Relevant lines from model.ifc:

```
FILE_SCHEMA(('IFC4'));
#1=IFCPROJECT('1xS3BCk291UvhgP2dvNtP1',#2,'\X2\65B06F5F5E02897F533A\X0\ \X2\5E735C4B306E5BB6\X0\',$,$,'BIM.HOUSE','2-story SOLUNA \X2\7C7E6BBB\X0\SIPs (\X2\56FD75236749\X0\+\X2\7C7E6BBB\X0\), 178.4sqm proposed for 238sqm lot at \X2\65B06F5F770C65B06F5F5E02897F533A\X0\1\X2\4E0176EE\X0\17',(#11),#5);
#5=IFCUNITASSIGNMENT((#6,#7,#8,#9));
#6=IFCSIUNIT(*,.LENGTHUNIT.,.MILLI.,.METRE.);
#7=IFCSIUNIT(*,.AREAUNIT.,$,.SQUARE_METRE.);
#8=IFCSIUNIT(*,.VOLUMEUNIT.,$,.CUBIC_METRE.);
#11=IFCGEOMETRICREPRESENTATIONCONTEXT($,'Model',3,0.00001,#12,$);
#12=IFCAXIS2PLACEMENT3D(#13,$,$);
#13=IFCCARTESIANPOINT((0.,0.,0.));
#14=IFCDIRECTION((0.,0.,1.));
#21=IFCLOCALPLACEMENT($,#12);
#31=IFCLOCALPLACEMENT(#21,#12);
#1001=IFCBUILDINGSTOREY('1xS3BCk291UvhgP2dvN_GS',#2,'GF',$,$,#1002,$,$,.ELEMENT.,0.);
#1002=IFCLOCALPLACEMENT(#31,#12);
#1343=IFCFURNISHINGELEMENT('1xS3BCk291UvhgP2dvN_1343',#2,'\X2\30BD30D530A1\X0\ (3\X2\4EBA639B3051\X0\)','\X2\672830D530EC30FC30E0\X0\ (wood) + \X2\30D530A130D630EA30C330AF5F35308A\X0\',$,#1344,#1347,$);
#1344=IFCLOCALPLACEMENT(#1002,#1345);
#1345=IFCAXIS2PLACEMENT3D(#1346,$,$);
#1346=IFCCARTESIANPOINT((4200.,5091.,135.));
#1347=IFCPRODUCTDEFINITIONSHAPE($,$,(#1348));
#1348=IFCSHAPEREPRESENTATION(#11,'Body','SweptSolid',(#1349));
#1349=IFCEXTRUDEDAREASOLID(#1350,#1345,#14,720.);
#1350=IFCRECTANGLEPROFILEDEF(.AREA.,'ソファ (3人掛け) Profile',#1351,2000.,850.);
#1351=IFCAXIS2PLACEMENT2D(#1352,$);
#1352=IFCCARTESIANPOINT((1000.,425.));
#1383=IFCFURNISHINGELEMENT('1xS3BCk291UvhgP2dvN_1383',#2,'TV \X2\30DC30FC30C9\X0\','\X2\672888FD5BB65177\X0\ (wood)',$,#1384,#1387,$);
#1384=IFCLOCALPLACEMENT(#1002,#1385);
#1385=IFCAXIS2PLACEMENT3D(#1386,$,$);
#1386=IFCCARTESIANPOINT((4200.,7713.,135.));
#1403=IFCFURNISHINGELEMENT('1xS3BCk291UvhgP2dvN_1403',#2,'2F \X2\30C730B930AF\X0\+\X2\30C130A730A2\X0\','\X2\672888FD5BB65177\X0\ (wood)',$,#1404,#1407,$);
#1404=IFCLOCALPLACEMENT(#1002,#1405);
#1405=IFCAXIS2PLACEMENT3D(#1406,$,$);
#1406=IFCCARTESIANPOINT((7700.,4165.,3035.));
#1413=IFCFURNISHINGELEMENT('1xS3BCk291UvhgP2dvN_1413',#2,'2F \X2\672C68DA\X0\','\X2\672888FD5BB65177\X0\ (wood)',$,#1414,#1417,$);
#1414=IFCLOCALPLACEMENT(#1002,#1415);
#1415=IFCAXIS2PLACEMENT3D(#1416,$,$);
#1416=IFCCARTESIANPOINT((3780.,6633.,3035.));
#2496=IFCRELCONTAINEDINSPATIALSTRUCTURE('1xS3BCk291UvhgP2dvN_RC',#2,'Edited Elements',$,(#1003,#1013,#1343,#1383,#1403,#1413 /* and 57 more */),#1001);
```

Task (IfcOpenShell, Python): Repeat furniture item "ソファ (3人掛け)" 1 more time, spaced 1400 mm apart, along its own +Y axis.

```python
import ifcopenshell
import ifcopenshell.api.geometry
import ifcopenshell.api.root
import ifcopenshell.util.element
import ifcopenshell.util.placement
import ifcopenshell.util.unit

model = ifcopenshell.open("model.ifc")
unit_scale = ifcopenshell.util.unit.calculate_unit_scale(model)


def reuse_history(source, copy):
    """copy_class also copies each property set's owner history, people and application; keep the originals."""
    for rel in copy.IsDefinedBy:
        if rel.is_a("IfcRelDefinesByProperties") and (history := rel.RelatingPropertyDefinition.OwnerHistory):
            rel.RelatingPropertyDefinition.OwnerHistory = source.OwnerHistory
            ifcopenshell.util.element.remove_deep2(model, history)


source = model.by_guid("1xS3BCk291UvhgP2dvN_1343")
base = ifcopenshell.util.placement.get_local_placement(source.ObjectPlacement)
step = base[:3, 1] * 1.4 / unit_scale

for i in range(1, 2):
    copy = ifcopenshell.api.root.copy_class(model, product=source)
    copy.Representation = ifcopenshell.util.element.copy_deep(
        model, source.Representation, exclude=["IfcGeometricRepresentationContext", "IfcRepresentationMap"]
    )
    reuse_history(source, copy)
    matrix = base.copy()
    matrix[:3, 3] += i * step
    print("added at", matrix[:3, 3].round(3) + 0.0)
    ifcopenshell.api.geometry.edit_object_placement(model, product=copy, matrix=matrix, is_si=False)

model.write("model-out.ifc")
```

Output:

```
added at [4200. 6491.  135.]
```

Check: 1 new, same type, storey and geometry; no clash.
